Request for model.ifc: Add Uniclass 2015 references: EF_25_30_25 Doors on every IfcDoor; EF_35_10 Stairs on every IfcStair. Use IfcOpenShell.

First a look at what the model holds.

```python
import ifcopenshell

model = ifcopenshell.open("model.ifc")
print(model.schema)
print("classifications:", [c.Name for c in model.by_type("IfcClassification")])
for ifc_class in ("IfcDoor", "IfcRoof", "IfcStair", "IfcWall", "IfcWindow"):
    print(ifc_class, len(model.by_type(ifc_class)))
```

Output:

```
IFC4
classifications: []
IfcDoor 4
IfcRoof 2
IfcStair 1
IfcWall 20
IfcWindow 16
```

```python
import ifcopenshell
import ifcopenshell.api.classification

model = ifcopenshell.open("model.ifc")

system = ifcopenshell.api.classification.add_classification(model, classification="Uniclass 2015")

codes = {
    "IfcDoor": ("EF_25_30_25", "Doors"),
    "IfcStair": ("EF_35_10", "Stairs"),
}
for ifc_class, (code, name) in codes.items():
    products = model.by_type(ifc_class)
    ifcopenshell.api.classification.add_reference(
        model, products=products, classification=system, identification=code, name=name
    )
    print(code, len(products))

model.write("model-out.ifc")
```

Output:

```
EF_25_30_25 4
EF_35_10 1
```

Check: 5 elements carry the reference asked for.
